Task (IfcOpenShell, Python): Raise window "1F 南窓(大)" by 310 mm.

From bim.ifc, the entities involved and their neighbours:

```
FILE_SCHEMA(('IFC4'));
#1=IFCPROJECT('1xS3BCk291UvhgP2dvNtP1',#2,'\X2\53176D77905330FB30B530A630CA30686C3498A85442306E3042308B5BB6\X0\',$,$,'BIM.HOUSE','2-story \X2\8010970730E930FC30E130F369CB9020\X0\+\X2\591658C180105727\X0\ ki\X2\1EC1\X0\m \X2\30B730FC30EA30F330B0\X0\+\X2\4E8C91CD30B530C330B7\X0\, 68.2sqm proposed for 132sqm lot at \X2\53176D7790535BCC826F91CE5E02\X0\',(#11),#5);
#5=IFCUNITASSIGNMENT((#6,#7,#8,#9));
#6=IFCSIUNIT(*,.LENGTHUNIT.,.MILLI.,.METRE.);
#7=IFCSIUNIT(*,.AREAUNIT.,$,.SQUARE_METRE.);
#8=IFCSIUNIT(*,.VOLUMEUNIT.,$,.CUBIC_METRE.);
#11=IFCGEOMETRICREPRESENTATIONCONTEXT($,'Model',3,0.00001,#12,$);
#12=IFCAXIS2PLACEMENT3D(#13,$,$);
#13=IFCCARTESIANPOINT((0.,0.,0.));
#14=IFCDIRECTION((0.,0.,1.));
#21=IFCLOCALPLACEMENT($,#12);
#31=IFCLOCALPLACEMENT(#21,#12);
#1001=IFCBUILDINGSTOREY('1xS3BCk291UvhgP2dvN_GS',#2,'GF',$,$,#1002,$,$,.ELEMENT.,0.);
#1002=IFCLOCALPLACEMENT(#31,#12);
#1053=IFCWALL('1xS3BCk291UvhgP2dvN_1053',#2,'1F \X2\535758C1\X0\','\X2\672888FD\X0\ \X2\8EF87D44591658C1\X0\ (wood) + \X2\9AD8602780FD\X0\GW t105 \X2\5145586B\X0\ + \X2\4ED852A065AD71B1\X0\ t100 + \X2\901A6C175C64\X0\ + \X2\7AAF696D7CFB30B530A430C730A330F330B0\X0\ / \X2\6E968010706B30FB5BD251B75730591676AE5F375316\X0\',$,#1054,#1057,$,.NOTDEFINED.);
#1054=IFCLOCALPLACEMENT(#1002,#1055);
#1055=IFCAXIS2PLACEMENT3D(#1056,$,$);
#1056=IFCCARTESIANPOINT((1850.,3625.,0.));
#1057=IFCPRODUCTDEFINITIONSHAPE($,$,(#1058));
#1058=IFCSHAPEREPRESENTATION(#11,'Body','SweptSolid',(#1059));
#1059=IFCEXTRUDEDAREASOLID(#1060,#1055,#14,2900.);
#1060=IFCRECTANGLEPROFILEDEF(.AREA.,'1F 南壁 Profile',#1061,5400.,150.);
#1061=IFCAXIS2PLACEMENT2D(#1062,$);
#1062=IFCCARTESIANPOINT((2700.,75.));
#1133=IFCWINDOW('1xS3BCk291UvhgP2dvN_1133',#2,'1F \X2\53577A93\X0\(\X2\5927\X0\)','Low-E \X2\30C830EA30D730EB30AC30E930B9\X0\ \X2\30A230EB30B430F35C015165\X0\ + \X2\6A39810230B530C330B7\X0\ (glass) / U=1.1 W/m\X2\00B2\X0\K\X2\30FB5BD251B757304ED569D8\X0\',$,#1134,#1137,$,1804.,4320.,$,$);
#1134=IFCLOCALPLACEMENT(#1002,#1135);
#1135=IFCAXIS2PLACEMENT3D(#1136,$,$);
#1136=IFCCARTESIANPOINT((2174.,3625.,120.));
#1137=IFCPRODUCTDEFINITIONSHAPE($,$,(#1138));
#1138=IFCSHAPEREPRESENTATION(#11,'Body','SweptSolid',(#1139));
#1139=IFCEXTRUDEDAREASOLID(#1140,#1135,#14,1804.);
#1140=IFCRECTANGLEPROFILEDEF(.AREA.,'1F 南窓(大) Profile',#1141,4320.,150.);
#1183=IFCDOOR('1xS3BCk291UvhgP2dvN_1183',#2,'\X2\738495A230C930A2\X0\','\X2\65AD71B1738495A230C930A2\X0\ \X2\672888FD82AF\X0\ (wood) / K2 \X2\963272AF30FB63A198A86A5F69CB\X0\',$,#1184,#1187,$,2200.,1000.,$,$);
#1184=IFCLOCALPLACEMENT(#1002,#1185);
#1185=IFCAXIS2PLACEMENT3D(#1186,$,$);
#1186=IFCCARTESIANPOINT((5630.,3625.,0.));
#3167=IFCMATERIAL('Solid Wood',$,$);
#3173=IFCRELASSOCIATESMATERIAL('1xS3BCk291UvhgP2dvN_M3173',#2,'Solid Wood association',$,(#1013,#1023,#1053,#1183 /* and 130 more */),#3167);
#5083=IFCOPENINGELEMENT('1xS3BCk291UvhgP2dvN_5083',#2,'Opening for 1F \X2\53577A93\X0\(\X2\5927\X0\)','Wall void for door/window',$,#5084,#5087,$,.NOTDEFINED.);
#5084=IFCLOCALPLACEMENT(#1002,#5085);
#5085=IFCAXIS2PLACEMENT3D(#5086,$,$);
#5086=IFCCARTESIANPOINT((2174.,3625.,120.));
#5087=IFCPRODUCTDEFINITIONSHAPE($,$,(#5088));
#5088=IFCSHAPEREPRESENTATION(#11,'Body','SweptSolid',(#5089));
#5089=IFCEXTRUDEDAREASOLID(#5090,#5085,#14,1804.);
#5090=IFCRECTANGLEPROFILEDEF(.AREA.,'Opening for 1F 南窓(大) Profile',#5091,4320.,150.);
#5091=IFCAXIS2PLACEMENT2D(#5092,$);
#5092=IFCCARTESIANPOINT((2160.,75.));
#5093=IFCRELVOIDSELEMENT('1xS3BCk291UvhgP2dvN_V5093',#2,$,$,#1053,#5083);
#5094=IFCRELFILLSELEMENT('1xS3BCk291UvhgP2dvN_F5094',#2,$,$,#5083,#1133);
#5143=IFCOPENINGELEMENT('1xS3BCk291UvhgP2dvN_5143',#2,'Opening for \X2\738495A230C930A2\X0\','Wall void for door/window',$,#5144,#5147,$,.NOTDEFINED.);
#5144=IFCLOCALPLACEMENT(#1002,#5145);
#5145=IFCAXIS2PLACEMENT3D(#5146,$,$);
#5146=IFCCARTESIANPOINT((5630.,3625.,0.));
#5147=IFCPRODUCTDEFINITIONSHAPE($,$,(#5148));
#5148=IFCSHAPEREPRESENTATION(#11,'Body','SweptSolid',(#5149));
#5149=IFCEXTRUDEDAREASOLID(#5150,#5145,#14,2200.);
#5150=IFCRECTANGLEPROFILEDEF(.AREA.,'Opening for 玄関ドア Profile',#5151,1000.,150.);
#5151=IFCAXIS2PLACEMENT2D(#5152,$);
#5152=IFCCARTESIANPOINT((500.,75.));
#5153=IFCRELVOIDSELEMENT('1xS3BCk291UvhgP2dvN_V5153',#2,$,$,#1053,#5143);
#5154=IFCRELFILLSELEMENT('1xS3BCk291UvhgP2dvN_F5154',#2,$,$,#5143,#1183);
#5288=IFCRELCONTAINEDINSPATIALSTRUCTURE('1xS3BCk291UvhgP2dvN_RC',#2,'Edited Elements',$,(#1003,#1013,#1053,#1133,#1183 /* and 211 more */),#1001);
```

```python
import numpy as np
import ifcopenshell
import ifcopenshell.api.geometry
import ifcopenshell.util.placement
import ifcopenshell.util.unit

model = ifcopenshell.open("bim.ifc")
unit_scale = ifcopenshell.util.unit.calculate_unit_scale(model)

window = model.by_id(1133)
opening = window.FillsVoids[0].RelatingOpeningElement
dz = 0.31 / unit_scale

shift = np.array([0.0, 0.0, dz])
# The window is not placed relative to its opening, so move both.
for product in (opening, window):
    matrix = ifcopenshell.util.placement.get_local_placement(product.ObjectPlacement)
    matrix[:3, 3] += shift
    ifcopenshell.api.geometry.edit_object_placement(model, product=product, matrix=matrix, is_si=False)

print(f"moved by {dz * unit_scale:+.3f} m")

model.write("bim_v2.ifc")
```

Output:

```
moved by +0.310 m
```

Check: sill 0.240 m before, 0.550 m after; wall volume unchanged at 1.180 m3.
